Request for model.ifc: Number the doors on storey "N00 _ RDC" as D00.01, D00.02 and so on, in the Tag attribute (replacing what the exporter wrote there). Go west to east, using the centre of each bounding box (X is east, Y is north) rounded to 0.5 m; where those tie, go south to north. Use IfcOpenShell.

First a look at what the model holds.

```python
import ifcopenshell
import ifcopenshell.util.element
import ifcopenshell.util.placement

model = ifcopenshell.open("model.ifc")
print(model.schema)
storey = next(s for s in model.by_type("IfcBuildingStorey") if s.Name == "N00 _ RDC")
doors = [e for e in ifcopenshell.util.element.get_decomposition(storey) if e.is_a("IfcDoor")]
for e in sorted(doors, key=lambda e: e.id()):
    origin = ifcopenshell.util.placement.get_local_placement(e.ObjectPlacement)[:3, 3]
    print(e.id(), e.Tag, e.Name, origin.round(2) + 0.0, sep=" | ")
```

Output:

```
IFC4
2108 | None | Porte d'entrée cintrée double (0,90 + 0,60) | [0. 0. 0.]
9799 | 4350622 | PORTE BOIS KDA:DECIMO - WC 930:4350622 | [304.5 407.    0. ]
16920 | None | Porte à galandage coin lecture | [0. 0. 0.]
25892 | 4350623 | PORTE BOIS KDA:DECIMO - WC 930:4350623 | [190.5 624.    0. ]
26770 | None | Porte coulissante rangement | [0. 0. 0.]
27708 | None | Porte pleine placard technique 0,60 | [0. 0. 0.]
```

```python
import ifcopenshell
import ifcopenshell.geom
import ifcopenshell.util.element
import ifcopenshell.util.shape

model = ifcopenshell.open("model.ifc")
settings = ifcopenshell.geom.settings()
settings.set("use-world-coords", True)


def centre(element):
    shape = ifcopenshell.geom.create_shape(settings, element)
    return ifcopenshell.util.shape.get_bbox_centroid(shape.geometry)


storey = next(s for s in model.by_type("IfcBuildingStorey") if s.Name == "N00 _ RDC")
doors = [e for e in ifcopenshell.util.element.get_decomposition(storey) if e.is_a("IfcDoor")]

# Insertion points can sit at a corner or the storey origin, so sort by the geometry (in metres).
centres = {e: centre(e) for e in doors}
doors.sort(key=lambda e: (round(centres[e][0] / 0.5), centres[e][1]))

for i, e in enumerate(doors, start=1):
    number = f"D00.{i:02d}"
    e.Tag = number
    print(e.id(), number)

model.write("model-out.ifc")
```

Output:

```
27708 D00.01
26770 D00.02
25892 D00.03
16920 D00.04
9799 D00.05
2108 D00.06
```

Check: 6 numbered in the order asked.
